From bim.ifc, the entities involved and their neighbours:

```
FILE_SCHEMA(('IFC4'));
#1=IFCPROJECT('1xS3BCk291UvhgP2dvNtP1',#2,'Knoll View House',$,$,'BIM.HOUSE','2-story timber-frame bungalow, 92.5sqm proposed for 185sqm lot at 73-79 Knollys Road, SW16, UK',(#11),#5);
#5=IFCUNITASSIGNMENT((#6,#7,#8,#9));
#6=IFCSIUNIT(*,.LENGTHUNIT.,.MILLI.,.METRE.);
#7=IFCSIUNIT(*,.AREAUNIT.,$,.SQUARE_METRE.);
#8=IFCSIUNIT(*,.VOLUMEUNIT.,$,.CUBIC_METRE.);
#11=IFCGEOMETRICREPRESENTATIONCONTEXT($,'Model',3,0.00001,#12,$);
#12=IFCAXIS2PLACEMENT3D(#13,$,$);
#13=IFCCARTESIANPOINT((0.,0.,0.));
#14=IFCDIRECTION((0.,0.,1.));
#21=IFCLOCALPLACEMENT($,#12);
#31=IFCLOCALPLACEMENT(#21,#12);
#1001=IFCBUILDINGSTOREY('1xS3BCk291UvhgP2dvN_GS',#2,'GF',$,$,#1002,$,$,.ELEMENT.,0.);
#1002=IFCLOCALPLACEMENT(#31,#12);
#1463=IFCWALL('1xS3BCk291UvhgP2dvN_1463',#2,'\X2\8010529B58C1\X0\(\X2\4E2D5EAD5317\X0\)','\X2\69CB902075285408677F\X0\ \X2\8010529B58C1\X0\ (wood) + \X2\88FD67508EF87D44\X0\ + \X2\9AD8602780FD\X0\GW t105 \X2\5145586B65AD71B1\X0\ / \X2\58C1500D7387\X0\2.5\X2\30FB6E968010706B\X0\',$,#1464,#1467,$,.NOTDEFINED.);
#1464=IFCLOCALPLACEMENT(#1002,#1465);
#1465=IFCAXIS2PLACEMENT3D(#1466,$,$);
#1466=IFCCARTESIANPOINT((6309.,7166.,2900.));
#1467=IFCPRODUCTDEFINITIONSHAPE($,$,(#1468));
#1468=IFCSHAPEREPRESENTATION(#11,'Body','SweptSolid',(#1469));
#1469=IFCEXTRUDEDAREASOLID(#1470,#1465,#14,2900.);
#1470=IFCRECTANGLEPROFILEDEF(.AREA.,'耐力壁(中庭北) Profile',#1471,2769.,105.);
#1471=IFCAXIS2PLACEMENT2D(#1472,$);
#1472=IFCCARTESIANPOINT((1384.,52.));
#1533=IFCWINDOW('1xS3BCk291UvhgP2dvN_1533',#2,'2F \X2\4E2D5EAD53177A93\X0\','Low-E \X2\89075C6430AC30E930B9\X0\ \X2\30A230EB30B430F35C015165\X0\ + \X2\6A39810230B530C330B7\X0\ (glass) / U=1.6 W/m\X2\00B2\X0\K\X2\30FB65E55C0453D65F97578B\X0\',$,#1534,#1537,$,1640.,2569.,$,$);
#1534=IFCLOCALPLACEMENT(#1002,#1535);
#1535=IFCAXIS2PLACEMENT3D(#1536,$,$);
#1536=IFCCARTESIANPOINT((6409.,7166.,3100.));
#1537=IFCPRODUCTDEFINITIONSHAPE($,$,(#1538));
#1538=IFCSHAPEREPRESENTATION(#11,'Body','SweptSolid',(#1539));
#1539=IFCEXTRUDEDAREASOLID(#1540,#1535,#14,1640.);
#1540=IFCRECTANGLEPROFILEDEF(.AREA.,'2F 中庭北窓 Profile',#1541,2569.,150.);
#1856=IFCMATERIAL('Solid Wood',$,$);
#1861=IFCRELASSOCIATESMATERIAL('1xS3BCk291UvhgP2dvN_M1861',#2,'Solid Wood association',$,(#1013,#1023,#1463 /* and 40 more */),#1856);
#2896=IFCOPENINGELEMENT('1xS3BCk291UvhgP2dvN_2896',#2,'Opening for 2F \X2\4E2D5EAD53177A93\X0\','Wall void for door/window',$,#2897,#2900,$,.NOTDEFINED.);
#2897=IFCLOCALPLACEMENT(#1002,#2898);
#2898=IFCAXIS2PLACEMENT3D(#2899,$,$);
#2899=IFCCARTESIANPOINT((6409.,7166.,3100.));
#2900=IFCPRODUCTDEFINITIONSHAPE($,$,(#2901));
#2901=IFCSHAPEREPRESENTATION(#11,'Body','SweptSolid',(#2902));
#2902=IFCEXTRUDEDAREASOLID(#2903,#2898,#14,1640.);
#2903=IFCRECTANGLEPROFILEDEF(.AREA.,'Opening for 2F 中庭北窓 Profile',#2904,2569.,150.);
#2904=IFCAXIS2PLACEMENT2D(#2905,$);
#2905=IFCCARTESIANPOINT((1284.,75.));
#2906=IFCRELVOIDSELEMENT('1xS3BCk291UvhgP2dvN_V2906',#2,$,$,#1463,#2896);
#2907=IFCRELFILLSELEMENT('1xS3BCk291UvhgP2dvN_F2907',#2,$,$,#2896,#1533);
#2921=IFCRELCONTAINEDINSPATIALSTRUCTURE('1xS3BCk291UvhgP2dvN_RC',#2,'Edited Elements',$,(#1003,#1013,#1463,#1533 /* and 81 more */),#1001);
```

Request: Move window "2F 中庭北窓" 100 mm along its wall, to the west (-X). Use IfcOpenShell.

```python
import ifcopenshell
import ifcopenshell.api.geometry
import ifcopenshell.util.placement

model = ifcopenshell.open("bim.ifc")

window = model.by_id(1533)
opening = window.FillsVoids[0].RelatingOpeningElement
wall = opening.VoidsElements[0].RelatingBuildingElement

wall_matrix = ifcopenshell.util.placement.get_local_placement(wall.ObjectPlacement)
shift = wall_matrix[:3, 0] * -100.0
before = ifcopenshell.util.placement.get_local_placement(window.ObjectPlacement)[:3, 3].copy()

# The window is not placed relative to its opening, so move both.
for product in (opening, window):
    matrix = ifcopenshell.util.placement.get_local_placement(product.ObjectPlacement)
    matrix[:3, 3] += shift
    ifcopenshell.api.geometry.edit_object_placement(model, product=product, matrix=matrix, is_si=False)

after = ifcopenshell.util.placement.get_local_placement(window.ObjectPlacement)[:3, 3]
print("window moved by", (after - before).round(3) + 0.0)

model.write("bim_updated.ifc")
```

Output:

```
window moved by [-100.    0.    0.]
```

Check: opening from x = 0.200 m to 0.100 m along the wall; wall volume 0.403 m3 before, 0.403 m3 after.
